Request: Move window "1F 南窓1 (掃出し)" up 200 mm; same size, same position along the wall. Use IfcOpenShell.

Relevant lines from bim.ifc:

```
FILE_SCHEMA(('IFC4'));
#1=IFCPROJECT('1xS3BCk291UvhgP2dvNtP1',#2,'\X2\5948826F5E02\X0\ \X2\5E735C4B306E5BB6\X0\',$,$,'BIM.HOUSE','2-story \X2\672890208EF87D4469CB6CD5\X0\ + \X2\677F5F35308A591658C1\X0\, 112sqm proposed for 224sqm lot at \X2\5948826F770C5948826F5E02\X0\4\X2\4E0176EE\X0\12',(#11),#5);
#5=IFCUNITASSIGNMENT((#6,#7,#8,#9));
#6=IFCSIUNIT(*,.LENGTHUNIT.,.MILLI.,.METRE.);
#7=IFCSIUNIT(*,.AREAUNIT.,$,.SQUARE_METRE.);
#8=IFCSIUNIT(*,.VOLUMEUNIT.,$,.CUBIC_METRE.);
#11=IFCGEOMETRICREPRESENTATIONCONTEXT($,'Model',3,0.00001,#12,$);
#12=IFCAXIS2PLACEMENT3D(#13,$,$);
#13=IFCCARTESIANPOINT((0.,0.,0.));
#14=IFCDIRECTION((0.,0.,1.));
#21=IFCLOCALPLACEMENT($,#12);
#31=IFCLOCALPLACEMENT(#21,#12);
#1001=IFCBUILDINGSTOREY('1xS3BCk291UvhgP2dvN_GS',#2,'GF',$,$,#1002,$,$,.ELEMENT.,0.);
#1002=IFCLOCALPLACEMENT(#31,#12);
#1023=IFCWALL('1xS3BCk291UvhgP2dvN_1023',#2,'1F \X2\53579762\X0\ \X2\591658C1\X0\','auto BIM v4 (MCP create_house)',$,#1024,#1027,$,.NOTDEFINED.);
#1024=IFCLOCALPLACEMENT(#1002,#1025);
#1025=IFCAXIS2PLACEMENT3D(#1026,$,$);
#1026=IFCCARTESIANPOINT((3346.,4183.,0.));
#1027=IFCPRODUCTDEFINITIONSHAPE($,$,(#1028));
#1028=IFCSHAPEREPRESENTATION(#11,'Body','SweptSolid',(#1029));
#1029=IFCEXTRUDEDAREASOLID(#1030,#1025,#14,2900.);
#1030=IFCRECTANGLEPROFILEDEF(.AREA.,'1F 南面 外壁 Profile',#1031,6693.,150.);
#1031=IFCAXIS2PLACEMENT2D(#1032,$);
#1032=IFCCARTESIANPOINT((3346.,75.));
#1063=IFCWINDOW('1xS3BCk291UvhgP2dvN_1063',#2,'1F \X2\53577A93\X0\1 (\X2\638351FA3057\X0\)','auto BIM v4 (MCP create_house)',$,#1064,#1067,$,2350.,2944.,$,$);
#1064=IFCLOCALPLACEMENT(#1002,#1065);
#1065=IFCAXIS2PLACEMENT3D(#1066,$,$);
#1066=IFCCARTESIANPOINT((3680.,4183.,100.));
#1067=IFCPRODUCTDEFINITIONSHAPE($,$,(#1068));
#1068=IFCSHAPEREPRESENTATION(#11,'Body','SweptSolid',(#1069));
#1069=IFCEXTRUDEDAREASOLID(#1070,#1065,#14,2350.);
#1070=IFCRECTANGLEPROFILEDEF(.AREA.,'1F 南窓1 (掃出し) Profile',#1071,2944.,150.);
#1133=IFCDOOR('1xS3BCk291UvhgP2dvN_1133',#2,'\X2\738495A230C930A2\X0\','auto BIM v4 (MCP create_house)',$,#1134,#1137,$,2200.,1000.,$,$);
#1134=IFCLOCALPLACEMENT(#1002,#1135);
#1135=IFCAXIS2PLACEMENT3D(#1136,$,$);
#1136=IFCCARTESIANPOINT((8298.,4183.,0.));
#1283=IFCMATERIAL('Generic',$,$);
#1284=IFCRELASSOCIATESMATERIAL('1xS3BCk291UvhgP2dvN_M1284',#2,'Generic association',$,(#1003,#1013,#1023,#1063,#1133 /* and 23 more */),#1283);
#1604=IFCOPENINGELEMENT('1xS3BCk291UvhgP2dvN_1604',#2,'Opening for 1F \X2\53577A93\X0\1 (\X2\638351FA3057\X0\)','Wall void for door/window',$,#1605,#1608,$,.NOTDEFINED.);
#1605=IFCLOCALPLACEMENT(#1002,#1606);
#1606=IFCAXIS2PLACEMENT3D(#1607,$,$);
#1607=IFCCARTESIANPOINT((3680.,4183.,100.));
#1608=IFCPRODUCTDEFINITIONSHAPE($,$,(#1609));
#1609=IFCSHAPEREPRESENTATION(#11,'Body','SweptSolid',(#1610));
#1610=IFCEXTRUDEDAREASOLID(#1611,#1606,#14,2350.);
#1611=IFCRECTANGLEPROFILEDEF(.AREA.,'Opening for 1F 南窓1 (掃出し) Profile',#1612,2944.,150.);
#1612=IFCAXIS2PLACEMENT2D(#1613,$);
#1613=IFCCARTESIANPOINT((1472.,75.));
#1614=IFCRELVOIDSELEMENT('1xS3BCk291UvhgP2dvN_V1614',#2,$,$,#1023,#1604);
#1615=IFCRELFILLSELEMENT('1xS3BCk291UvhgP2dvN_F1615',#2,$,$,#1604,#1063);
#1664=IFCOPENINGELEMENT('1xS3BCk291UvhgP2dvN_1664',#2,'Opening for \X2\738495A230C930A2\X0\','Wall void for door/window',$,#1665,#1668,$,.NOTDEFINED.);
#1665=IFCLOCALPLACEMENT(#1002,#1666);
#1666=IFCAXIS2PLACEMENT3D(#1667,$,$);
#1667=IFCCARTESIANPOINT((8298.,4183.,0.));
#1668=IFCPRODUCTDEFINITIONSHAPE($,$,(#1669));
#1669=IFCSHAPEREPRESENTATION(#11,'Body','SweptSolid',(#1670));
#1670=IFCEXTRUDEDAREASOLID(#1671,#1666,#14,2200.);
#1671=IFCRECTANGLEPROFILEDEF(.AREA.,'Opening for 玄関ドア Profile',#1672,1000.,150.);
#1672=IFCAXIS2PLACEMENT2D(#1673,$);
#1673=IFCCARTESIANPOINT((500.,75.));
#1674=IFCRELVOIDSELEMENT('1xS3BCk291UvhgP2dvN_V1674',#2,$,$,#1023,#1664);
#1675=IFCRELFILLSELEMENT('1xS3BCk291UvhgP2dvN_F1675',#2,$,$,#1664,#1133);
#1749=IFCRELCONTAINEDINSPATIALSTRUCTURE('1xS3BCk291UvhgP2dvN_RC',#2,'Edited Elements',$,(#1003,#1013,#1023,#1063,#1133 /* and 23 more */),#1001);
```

```python
import numpy as np
import ifcopenshell
import ifcopenshell.api.geometry
import ifcopenshell.util.placement
import ifcopenshell.util.unit

model = ifcopenshell.open("bim.ifc")
unit_scale = ifcopenshell.util.unit.calculate_unit_scale(model)

window = model.by_id(1063)
opening = window.FillsVoids[0].RelatingOpeningElement
dz = 200.0

shift = np.array([0.0, 0.0, dz])
# The window is not placed relative to its opening, so move both.
for product in (opening, window):
    matrix = ifcopenshell.util.placement.get_local_placement(product.ObjectPlacement)
    matrix[:3, 3] += shift
    ifcopenshell.api.geometry.edit_object_placement(model, product=product, matrix=matrix, is_si=False)

print(f"moved by {dz * unit_scale:+.3f} m")

model.write("bim_updated.ifc")
```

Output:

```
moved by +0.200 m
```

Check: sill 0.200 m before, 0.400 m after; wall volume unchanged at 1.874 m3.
